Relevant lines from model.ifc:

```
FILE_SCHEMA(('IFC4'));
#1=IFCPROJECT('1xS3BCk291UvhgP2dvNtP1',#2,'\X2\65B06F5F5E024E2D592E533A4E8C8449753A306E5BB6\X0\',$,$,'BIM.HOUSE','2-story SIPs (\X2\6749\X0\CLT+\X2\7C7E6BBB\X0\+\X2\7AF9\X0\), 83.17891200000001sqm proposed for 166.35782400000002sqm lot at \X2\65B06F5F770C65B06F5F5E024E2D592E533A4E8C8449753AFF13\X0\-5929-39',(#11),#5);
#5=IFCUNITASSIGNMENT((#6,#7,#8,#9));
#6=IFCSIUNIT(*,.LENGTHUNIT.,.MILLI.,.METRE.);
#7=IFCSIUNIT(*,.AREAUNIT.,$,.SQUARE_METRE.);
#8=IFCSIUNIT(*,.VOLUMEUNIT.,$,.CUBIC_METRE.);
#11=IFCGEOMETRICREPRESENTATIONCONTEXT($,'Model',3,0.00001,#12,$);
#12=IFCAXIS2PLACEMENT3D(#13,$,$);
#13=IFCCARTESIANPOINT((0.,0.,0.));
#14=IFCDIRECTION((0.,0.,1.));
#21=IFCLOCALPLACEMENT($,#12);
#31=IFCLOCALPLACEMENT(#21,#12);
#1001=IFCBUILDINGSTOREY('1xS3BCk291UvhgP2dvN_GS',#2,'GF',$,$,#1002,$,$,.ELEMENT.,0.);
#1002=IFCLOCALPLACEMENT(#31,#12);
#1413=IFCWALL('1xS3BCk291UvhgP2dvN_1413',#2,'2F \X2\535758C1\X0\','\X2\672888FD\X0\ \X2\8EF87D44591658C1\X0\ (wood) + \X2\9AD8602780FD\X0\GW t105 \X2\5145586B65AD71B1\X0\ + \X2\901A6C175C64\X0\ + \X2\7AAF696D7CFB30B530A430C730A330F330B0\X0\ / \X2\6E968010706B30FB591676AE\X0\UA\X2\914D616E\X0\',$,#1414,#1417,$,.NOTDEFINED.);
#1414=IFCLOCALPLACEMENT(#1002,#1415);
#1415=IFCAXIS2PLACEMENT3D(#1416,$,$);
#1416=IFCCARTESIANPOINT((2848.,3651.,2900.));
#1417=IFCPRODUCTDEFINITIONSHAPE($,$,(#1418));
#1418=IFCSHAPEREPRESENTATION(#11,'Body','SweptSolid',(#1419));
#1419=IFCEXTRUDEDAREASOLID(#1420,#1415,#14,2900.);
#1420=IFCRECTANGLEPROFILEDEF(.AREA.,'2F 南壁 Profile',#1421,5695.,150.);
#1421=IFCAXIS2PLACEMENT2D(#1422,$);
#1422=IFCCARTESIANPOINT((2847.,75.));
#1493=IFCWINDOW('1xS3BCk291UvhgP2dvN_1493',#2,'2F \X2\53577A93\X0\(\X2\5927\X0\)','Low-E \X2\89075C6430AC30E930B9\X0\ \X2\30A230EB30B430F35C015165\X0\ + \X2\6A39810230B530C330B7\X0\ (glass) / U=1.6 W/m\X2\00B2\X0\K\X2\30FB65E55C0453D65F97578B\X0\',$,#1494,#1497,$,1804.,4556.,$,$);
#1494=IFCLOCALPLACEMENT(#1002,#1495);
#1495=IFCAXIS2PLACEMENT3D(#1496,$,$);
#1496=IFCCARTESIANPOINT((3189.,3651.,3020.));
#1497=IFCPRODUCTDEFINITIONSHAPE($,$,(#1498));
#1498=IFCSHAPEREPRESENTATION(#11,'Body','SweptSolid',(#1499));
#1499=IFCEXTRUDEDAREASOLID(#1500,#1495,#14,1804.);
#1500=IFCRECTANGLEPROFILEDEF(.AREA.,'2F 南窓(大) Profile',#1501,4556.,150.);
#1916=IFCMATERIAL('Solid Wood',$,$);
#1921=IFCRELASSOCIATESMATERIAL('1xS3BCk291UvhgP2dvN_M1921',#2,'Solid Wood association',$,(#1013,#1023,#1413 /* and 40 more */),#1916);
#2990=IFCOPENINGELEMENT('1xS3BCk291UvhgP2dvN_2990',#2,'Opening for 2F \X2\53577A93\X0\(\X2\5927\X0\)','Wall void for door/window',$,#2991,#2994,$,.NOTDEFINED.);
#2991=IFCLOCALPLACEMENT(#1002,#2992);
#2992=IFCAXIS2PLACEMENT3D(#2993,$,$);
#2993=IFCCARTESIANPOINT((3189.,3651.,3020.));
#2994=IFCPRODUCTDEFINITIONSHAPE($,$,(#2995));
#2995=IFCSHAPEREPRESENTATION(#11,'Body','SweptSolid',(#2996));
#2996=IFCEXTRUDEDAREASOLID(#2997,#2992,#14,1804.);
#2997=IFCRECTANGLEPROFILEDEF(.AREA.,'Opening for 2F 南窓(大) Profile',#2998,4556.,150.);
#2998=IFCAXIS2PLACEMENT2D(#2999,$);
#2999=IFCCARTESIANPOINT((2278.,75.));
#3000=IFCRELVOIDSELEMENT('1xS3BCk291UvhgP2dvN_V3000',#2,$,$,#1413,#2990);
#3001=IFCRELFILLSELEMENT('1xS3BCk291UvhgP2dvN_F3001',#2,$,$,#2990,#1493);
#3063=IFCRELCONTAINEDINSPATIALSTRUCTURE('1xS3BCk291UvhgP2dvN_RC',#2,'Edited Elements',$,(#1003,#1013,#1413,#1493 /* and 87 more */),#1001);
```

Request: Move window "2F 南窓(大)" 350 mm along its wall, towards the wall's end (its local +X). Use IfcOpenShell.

```python
import ifcopenshell
import ifcopenshell.api.geometry
import ifcopenshell.util.placement

model = ifcopenshell.open("model.ifc")

window = model.by_guid("1xS3BCk291UvhgP2dvN_1493")
opening = window.FillsVoids[0].RelatingOpeningElement
wall = opening.VoidsElements[0].RelatingBuildingElement

wall_matrix = ifcopenshell.util.placement.get_local_placement(wall.ObjectPlacement)
shift = wall_matrix[:3, 0] * 350.0
before = ifcopenshell.util.placement.get_local_placement(window.ObjectPlacement)[:3, 3].copy()

# The window is not placed relative to its opening, so move both.
for product in (opening, window):
    matrix = ifcopenshell.util.placement.get_local_placement(product.ObjectPlacement)
    matrix[:3, 3] += shift
    ifcopenshell.api.geometry.edit_object_placement(model, product=product, matrix=matrix, is_si=False)

after = ifcopenshell.util.placement.get_local_placement(window.ObjectPlacement)[:3, 3]
print("window moved by", (after - before).round(3) + 0.0)

model.write("model_edited.ifc")
```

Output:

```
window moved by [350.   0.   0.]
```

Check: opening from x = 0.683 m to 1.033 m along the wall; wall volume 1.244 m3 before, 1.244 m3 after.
